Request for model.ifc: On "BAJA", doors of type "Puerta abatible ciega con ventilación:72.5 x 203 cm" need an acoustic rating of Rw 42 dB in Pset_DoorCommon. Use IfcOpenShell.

First a look at what the model holds.

```python
import ifcopenshell
import ifcopenshell.util.element

model = ifcopenshell.open("model.ifc")
print(model.schema)
storey = next(s for s in model.by_type("IfcBuildingStorey") if s.Name == "BAJA")
doors = [e for e in ifcopenshell.util.element.get_decomposition(storey) if e.is_a("IfcDoor")]
seen = {}
for e in doors:
    element_type = ifcopenshell.util.element.get_type(e)
    key = (element_type.Name if element_type != e and element_type else None, ifcopenshell.util.element.get_pset(e, "Pset_DoorCommon", "AcousticRating"))
    seen[key] = seen.get(key, 0) + 1
for (name, value), count in sorted(seen.items(), key=str):
    print(count, "x", name, "|", value)
```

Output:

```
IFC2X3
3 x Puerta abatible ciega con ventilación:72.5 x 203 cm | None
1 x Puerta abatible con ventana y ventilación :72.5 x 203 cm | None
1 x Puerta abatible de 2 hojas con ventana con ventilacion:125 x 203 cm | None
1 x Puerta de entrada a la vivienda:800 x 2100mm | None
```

```python
import ifcopenshell
import ifcopenshell.api.pset
import ifcopenshell.util.element

model = ifcopenshell.open("model.ifc")

storey = next(s for s in model.by_type("IfcBuildingStorey") if s.Name == "BAJA")
doors = [e for e in ifcopenshell.util.element.get_decomposition(storey) if e.is_a("IfcDoor")]

count = 0
for e in doors:
    element_type = ifcopenshell.util.element.get_type(e)
    if element_type in (None, e) or element_type.Name != "Puerta abatible ciega con ventilación:72.5 x 203 cm":
        continue
    # add_pset returns the element's existing set when there is one.
    pset = ifcopenshell.api.pset.add_pset(model, product=e, name="Pset_DoorCommon")
    ifcopenshell.api.pset.edit_pset(model, pset=pset, properties={"AcousticRating": "Rw 42 dB"})
    count += 1

print(count, "doors updated")

model.write("model_edited.ifc")
```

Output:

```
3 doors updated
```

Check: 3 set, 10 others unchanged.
